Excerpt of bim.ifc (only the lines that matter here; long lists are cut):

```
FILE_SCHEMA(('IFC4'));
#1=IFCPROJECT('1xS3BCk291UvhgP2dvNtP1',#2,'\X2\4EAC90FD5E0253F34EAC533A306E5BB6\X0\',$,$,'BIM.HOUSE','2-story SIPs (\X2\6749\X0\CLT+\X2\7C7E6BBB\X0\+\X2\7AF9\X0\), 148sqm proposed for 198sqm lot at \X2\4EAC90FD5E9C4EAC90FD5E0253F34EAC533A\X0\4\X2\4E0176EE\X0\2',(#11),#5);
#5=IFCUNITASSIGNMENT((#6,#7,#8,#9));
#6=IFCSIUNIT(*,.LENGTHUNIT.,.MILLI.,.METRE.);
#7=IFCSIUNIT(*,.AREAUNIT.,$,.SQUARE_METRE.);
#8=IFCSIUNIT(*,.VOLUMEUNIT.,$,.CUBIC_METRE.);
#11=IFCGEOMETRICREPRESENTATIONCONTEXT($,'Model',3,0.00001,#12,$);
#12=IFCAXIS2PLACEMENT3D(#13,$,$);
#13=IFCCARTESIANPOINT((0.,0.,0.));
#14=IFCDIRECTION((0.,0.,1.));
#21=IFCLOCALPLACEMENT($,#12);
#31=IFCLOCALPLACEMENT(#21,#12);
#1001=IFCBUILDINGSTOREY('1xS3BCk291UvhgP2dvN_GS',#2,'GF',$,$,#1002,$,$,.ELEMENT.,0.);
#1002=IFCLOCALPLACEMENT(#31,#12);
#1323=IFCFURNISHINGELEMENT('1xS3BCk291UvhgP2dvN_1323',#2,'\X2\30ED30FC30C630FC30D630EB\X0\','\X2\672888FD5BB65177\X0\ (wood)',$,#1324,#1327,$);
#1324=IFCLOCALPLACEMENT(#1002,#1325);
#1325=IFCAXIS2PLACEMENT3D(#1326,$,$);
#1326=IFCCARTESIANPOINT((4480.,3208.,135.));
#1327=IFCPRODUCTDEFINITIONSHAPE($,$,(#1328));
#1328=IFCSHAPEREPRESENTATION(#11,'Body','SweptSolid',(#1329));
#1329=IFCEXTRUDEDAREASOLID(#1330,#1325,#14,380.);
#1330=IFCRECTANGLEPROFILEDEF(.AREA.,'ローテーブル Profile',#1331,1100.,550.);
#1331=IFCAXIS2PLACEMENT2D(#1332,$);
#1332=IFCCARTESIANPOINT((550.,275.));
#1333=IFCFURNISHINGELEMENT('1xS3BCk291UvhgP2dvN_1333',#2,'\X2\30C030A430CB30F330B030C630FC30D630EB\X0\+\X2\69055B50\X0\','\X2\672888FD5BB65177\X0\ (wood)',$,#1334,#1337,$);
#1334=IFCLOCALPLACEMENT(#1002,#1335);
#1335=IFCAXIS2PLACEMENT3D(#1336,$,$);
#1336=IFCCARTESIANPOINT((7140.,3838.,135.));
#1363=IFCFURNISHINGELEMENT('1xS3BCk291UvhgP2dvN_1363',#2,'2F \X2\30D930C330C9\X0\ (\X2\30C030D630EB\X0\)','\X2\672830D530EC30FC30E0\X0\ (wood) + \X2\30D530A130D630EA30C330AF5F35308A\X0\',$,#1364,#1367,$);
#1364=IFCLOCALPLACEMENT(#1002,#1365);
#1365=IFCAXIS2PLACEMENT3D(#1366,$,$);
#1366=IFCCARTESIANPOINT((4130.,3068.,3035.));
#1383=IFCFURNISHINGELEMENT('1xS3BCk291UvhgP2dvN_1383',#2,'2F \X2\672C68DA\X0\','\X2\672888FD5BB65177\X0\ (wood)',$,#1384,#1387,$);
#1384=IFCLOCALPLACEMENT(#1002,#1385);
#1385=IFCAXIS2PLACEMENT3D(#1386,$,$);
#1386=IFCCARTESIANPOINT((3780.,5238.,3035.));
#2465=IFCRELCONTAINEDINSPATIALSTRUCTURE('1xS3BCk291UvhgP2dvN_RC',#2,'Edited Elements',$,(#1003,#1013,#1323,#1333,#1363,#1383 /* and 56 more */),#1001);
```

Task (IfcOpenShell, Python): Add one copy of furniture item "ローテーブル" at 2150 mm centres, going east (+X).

```python
import numpy as np
import ifcopenshell
import ifcopenshell.api.geometry
import ifcopenshell.api.root
import ifcopenshell.util.element
import ifcopenshell.util.placement
import ifcopenshell.util.unit

model = ifcopenshell.open("bim.ifc")
unit_scale = ifcopenshell.util.unit.calculate_unit_scale(model)


def reuse_history(source, copy):
    """copy_class also copies each property set's owner history, people and application; keep the originals."""
    for rel in copy.IsDefinedBy:
        if rel.is_a("IfcRelDefinesByProperties") and (history := rel.RelatingPropertyDefinition.OwnerHistory):
            rel.RelatingPropertyDefinition.OwnerHistory = source.OwnerHistory
            ifcopenshell.util.element.remove_deep2(model, history)


source = model.by_guid("1xS3BCk291UvhgP2dvN_1323")
base = ifcopenshell.util.placement.get_local_placement(source.ObjectPlacement)
step = np.array([1.0, 0.0, 0.0]) * 2.15 / unit_scale

for i in range(1, 2):
    copy = ifcopenshell.api.root.copy_class(model, product=source)
    copy.Representation = ifcopenshell.util.element.copy_deep(
        model, source.Representation, exclude=["IfcGeometricRepresentationContext", "IfcRepresentationMap"]
    )
    reuse_history(source, copy)
    matrix = base.copy()
    matrix[:3, 3] += i * step
    print("added at", matrix[:3, 3].round(3) + 0.0)
    ifcopenshell.api.geometry.edit_object_placement(model, product=copy, matrix=matrix, is_si=False)

model.write("bim_edited.ifc")
```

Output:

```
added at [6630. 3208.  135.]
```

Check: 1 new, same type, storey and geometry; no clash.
